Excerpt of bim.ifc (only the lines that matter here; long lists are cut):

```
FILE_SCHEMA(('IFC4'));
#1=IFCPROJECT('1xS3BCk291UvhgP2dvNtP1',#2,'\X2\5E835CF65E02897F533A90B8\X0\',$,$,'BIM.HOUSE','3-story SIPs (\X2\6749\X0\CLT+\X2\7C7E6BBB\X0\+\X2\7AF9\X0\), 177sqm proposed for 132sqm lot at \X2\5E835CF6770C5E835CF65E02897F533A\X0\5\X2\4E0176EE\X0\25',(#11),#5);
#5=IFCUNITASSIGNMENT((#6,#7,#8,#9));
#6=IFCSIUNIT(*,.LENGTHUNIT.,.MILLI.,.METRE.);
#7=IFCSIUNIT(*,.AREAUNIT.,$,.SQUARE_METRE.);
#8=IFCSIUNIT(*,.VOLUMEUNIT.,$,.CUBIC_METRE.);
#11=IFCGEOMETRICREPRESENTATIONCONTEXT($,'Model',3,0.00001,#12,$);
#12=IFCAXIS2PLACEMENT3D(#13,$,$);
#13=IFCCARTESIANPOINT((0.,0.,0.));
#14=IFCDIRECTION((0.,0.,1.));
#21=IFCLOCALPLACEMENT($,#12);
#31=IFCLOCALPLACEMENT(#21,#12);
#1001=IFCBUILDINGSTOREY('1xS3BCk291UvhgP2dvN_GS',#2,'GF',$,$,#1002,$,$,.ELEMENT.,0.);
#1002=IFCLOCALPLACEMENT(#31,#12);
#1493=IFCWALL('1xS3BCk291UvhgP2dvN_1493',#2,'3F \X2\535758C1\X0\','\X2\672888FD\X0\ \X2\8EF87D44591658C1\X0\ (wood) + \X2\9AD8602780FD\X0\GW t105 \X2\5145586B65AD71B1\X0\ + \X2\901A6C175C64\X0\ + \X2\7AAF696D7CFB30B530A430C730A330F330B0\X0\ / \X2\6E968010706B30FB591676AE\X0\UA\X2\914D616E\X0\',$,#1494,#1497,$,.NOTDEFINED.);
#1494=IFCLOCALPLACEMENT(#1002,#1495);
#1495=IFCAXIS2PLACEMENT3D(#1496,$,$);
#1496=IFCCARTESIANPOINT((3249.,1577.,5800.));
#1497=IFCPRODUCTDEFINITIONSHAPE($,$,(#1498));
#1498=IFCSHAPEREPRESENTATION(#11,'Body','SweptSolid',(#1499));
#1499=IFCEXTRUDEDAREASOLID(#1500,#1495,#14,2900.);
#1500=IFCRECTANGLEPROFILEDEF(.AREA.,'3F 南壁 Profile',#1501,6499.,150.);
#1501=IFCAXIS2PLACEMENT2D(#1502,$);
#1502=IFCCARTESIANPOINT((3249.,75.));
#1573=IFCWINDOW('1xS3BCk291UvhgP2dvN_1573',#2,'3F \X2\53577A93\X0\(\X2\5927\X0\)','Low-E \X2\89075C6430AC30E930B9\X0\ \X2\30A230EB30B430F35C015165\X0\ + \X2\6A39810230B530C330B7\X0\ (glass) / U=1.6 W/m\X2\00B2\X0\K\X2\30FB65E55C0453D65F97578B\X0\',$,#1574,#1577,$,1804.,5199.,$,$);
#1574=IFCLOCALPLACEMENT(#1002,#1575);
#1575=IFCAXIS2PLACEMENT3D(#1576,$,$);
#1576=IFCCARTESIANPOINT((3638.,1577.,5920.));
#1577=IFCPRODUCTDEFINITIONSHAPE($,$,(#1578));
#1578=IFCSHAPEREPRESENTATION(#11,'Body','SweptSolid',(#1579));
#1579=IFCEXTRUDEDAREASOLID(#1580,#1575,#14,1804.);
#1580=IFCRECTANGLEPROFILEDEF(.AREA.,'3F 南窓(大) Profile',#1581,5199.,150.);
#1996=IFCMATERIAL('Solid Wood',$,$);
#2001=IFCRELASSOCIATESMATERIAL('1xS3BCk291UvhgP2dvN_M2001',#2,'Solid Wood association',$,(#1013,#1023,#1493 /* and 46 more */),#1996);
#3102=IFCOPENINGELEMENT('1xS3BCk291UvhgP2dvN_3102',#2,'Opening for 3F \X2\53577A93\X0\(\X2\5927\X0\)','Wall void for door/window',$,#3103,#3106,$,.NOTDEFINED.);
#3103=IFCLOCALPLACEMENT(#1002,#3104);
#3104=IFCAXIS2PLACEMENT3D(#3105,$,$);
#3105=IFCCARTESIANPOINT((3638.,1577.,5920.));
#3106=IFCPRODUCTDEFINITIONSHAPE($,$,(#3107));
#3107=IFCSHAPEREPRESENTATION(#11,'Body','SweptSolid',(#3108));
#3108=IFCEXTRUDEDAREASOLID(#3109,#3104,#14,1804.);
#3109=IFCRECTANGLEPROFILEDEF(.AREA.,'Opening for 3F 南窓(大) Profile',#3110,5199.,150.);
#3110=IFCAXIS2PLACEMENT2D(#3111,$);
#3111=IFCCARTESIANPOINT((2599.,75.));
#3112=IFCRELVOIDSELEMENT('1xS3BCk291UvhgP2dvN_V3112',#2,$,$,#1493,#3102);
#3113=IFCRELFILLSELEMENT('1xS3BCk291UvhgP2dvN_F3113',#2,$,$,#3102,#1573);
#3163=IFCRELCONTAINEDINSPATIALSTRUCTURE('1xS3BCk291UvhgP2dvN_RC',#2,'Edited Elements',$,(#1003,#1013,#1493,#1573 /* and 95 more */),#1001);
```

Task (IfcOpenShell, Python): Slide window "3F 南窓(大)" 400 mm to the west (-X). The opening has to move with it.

```python
import ifcopenshell
import ifcopenshell.api.geometry
import ifcopenshell.util.placement
import ifcopenshell.util.unit

model = ifcopenshell.open("bim.ifc")
unit_scale = ifcopenshell.util.unit.calculate_unit_scale(model)

window = model.by_guid("1xS3BCk291UvhgP2dvN_1573")
opening = window.FillsVoids[0].RelatingOpeningElement
wall = opening.VoidsElements[0].RelatingBuildingElement

wall_matrix = ifcopenshell.util.placement.get_local_placement(wall.ObjectPlacement)
shift = wall_matrix[:3, 0] * -0.4 / unit_scale
before = ifcopenshell.util.placement.get_local_placement(window.ObjectPlacement)[:3, 3].copy()

# The window is not placed relative to its opening, so move both.
for product in (opening, window):
    matrix = ifcopenshell.util.placement.get_local_placement(product.ObjectPlacement)
    matrix[:3, 3] += shift
    ifcopenshell.api.geometry.edit_object_placement(model, product=product, matrix=matrix, is_si=False)

after = ifcopenshell.util.placement.get_local_placement(window.ObjectPlacement)[:3, 3]
print("window moved by", (after - before).round(3) + 0.0)

model.write("bim_v2.ifc")
```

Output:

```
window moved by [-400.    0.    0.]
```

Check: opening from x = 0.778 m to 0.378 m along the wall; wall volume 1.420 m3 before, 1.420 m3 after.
